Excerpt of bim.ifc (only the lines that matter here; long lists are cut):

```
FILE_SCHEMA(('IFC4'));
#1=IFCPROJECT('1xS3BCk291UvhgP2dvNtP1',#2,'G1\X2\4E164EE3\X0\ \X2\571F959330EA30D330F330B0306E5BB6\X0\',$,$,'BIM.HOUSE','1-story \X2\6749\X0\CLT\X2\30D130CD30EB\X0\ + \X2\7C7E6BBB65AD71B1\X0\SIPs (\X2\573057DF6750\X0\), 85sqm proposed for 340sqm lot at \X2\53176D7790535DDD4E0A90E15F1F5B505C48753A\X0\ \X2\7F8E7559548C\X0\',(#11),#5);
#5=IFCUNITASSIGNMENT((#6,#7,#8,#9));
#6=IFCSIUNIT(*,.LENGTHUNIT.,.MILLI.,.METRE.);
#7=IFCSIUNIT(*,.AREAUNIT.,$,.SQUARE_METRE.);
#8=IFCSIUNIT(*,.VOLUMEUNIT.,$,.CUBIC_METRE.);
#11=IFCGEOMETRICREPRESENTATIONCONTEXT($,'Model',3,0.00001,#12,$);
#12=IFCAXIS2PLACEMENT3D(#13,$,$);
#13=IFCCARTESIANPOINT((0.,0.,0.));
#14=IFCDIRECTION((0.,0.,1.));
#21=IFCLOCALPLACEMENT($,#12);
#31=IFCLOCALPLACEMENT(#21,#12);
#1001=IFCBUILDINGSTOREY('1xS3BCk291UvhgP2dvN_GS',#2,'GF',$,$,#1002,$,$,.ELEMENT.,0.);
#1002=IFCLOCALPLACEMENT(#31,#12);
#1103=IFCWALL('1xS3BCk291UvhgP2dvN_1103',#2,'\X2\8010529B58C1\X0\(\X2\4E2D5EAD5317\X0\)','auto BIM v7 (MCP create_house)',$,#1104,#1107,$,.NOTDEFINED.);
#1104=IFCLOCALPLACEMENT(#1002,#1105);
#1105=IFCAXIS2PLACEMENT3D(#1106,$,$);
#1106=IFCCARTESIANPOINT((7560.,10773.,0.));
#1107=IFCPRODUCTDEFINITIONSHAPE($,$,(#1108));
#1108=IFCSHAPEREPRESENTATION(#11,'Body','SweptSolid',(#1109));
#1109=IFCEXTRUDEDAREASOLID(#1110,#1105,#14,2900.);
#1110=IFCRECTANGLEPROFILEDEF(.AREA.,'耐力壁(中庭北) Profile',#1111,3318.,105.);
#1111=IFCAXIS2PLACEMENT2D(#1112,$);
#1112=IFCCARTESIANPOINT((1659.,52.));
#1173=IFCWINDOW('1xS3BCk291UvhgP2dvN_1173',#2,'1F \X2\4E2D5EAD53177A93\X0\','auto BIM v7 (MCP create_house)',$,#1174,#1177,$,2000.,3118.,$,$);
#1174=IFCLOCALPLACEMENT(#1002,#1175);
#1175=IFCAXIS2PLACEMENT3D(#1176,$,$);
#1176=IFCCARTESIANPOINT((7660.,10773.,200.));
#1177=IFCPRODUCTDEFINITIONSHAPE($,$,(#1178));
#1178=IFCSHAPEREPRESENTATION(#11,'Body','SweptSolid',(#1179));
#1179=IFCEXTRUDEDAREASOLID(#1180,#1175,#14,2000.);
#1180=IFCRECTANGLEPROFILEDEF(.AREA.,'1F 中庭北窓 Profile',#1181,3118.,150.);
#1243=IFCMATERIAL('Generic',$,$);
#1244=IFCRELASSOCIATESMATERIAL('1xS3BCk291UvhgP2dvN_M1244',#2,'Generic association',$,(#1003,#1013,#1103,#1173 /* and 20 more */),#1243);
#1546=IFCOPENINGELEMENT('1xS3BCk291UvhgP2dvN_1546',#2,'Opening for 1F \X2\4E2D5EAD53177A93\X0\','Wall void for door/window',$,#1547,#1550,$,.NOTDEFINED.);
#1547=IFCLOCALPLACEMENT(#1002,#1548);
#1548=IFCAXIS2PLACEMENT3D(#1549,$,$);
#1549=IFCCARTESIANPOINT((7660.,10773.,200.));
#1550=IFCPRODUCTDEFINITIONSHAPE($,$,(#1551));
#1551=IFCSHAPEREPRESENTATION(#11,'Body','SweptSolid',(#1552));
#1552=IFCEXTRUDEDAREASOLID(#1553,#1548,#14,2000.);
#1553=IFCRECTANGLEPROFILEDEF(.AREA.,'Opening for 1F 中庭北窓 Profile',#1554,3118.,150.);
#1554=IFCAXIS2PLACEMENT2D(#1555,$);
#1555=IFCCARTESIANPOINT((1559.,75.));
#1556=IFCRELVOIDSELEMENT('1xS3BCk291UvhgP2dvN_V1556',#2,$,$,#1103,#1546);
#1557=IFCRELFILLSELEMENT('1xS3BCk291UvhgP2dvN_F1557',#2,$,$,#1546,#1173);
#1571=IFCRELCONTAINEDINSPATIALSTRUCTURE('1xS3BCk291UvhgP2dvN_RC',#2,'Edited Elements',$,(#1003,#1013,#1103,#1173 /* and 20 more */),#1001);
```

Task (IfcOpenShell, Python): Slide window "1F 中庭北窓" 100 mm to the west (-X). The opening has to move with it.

```python
import ifcopenshell
import ifcopenshell.api.geometry
import ifcopenshell.util.placement
import ifcopenshell.util.unit

model = ifcopenshell.open("bim.ifc")
unit_scale = ifcopenshell.util.unit.calculate_unit_scale(model)

window = model.by_guid("1xS3BCk291UvhgP2dvN_1173")
opening = window.FillsVoids[0].RelatingOpeningElement
wall = opening.VoidsElements[0].RelatingBuildingElement

wall_matrix = ifcopenshell.util.placement.get_local_placement(wall.ObjectPlacement)
shift = wall_matrix[:3, 0] * -0.1 / unit_scale
before = ifcopenshell.util.placement.get_local_placement(window.ObjectPlacement)[:3, 3].copy()

# The window is not placed relative to its opening, so move both.
for product in (opening, window):
    matrix = ifcopenshell.util.placement.get_local_placement(product.ObjectPlacement)
    matrix[:3, 3] += shift
    ifcopenshell.api.geometry.edit_object_placement(model, product=product, matrix=matrix, is_si=False)

after = ifcopenshell.util.placement.get_local_placement(window.ObjectPlacement)[:3, 3]
print("window moved by", (after - before).round(3) + 0.0)

model.write("bim_edited.ifc")
```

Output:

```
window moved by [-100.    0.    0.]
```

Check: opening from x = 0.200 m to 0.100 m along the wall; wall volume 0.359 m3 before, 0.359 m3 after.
